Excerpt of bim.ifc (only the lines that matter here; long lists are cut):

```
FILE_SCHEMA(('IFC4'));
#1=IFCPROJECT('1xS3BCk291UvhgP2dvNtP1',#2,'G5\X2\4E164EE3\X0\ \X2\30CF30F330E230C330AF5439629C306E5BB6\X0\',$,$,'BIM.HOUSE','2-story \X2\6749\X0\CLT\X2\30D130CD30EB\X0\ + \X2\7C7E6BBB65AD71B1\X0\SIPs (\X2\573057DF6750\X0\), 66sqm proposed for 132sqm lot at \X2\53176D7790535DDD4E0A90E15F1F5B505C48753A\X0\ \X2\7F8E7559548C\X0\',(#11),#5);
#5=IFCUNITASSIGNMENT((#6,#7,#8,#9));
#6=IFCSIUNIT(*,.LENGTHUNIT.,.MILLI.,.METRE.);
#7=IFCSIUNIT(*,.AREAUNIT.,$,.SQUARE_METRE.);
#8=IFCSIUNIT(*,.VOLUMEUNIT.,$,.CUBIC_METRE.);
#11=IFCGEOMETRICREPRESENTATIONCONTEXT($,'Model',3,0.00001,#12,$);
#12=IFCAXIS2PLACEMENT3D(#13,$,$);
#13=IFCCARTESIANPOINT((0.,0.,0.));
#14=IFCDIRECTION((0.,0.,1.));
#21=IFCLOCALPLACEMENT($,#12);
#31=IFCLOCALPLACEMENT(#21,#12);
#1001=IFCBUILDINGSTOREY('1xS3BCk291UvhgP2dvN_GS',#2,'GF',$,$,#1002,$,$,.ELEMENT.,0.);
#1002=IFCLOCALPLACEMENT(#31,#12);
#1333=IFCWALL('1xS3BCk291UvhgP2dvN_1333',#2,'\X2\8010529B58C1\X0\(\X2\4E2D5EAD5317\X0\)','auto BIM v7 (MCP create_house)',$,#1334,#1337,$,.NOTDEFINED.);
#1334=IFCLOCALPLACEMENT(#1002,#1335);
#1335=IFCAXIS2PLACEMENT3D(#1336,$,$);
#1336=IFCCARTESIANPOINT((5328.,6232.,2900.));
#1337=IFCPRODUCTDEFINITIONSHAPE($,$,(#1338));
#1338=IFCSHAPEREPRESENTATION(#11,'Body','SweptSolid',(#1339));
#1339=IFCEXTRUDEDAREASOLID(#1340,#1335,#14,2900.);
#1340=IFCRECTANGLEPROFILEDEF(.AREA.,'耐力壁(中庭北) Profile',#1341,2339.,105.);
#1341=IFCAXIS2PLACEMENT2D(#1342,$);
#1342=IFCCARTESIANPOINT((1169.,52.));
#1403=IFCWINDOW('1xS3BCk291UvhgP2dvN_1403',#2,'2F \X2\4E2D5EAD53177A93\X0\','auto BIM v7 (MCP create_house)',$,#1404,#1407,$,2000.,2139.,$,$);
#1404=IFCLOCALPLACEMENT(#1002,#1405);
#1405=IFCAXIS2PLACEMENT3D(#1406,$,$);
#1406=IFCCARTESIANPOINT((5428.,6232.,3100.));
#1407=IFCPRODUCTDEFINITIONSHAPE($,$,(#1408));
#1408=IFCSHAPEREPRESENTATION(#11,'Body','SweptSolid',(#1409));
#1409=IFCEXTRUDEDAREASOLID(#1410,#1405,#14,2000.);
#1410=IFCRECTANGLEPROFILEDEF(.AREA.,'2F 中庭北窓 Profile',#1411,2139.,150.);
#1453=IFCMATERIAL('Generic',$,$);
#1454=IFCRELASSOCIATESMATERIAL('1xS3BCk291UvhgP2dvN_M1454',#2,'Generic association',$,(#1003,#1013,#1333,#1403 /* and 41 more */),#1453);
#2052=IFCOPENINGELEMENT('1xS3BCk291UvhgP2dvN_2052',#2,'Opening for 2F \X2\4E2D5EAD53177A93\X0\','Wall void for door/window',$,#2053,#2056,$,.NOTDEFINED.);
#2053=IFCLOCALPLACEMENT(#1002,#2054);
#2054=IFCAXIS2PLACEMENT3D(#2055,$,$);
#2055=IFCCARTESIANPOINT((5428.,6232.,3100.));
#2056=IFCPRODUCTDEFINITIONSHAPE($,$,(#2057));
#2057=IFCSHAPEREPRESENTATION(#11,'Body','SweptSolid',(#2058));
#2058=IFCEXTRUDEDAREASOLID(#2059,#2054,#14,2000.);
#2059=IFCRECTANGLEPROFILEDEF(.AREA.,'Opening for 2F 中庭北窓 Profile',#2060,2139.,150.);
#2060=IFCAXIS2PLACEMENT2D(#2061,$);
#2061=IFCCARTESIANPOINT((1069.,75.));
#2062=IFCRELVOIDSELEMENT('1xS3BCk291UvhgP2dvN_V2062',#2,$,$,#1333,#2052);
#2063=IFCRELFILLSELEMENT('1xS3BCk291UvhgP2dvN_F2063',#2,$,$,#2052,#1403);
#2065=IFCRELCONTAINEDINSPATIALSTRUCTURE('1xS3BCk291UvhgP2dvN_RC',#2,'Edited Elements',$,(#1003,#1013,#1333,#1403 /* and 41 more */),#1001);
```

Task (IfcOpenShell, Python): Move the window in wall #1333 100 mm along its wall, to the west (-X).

```python
import ifcopenshell
import ifcopenshell.api.geometry
import ifcopenshell.util.placement

model = ifcopenshell.open("bim.ifc")

window = model.by_guid("1xS3BCk291UvhgP2dvN_1403")
opening = window.FillsVoids[0].RelatingOpeningElement
wall = opening.VoidsElements[0].RelatingBuildingElement

wall_matrix = ifcopenshell.util.placement.get_local_placement(wall.ObjectPlacement)
shift = wall_matrix[:3, 0] * -100.0
before = ifcopenshell.util.placement.get_local_placement(window.ObjectPlacement)[:3, 3].copy()

# The window is not placed relative to its opening, so move both.
for product in (opening, window):
    matrix = ifcopenshell.util.placement.get_local_placement(product.ObjectPlacement)
    matrix[:3, 3] += shift
    ifcopenshell.api.geometry.edit_object_placement(model, product=product, matrix=matrix, is_si=False)

after = ifcopenshell.util.placement.get_local_placement(window.ObjectPlacement)[:3, 3]
print("window moved by", (after - before).round(3) + 0.0)

model.write("bim-out.ifc")
```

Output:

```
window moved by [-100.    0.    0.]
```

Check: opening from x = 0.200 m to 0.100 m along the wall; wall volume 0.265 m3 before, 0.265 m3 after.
